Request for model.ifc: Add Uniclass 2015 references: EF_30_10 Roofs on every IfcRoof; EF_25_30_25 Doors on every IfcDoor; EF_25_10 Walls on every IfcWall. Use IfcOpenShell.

First a look at what the model holds.

```python
import ifcopenshell

model = ifcopenshell.open("model.ifc")
print(model.schema)
print("classifications:", [c.Name for c in model.by_type("IfcClassification")])
for ifc_class in ("IfcDoor", "IfcRoof", "IfcStair", "IfcWall", "IfcWindow"):
    print(ifc_class, len(model.by_type(ifc_class)))
```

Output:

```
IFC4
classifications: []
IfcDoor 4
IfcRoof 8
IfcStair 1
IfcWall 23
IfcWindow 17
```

```python
import ifcopenshell
import ifcopenshell.api.classification

model = ifcopenshell.open("model.ifc")

system = ifcopenshell.api.classification.add_classification(model, classification="Uniclass 2015")

codes = {
    "IfcRoof": ("EF_30_10", "Roofs"),
    "IfcDoor": ("EF_25_30_25", "Doors"),
    "IfcWall": ("EF_25_10", "Walls"),
}
for ifc_class, (code, name) in codes.items():
    products = model.by_type(ifc_class)
    ifcopenshell.api.classification.add_reference(
        model, products=products, classification=system, identification=code, name=name
    )
    print(code, len(products))

model.write("model_rev.ifc")
```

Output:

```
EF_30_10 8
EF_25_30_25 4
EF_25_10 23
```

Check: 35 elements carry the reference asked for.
